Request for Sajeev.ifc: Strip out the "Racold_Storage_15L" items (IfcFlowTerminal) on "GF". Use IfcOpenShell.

First a look at what the model holds.

```python
import ifcopenshell
import ifcopenshell.util.element

model = ifcopenshell.open("Sajeev.ifc")
print(model.schema)
storey = next(s for s in model.by_type("IfcBuildingStorey") if s.Name == "GF")
terminals = [e for e in ifcopenshell.util.element.get_decomposition(storey) if e.is_a("IfcFlowTerminal")]
seen = {}
for e in terminals:
    element_type = ifcopenshell.util.element.get_type(e)
    name = element_type.Name if element_type not in (None, e) else None
    seen[name] = seen.get(name, 0) + 1
for name, count in sorted(seen.items(), key=str):
    print(count, "x", name)
```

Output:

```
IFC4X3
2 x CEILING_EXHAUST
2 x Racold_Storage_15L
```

```python
import ifcopenshell
import ifcopenshell.api.root
import ifcopenshell.util.element

model = ifcopenshell.open("Sajeev.ifc")

storey = next(s for s in model.by_type("IfcBuildingStorey") if s.Name == "GF")
terminals = [e for e in ifcopenshell.util.element.get_decomposition(storey) if e.is_a("IfcFlowTerminal")]
targets = [e for e in terminals if (t := ifcopenshell.util.element.get_type(e)) not in (None, e) and t.Name == "Racold_Storage_15L"]

for e in targets:
    ifcopenshell.api.root.remove_product(model, product=e)
print(len(targets), "removed")

model.write("Sajeev_v2.ifc")
```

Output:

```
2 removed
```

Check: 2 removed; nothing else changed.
